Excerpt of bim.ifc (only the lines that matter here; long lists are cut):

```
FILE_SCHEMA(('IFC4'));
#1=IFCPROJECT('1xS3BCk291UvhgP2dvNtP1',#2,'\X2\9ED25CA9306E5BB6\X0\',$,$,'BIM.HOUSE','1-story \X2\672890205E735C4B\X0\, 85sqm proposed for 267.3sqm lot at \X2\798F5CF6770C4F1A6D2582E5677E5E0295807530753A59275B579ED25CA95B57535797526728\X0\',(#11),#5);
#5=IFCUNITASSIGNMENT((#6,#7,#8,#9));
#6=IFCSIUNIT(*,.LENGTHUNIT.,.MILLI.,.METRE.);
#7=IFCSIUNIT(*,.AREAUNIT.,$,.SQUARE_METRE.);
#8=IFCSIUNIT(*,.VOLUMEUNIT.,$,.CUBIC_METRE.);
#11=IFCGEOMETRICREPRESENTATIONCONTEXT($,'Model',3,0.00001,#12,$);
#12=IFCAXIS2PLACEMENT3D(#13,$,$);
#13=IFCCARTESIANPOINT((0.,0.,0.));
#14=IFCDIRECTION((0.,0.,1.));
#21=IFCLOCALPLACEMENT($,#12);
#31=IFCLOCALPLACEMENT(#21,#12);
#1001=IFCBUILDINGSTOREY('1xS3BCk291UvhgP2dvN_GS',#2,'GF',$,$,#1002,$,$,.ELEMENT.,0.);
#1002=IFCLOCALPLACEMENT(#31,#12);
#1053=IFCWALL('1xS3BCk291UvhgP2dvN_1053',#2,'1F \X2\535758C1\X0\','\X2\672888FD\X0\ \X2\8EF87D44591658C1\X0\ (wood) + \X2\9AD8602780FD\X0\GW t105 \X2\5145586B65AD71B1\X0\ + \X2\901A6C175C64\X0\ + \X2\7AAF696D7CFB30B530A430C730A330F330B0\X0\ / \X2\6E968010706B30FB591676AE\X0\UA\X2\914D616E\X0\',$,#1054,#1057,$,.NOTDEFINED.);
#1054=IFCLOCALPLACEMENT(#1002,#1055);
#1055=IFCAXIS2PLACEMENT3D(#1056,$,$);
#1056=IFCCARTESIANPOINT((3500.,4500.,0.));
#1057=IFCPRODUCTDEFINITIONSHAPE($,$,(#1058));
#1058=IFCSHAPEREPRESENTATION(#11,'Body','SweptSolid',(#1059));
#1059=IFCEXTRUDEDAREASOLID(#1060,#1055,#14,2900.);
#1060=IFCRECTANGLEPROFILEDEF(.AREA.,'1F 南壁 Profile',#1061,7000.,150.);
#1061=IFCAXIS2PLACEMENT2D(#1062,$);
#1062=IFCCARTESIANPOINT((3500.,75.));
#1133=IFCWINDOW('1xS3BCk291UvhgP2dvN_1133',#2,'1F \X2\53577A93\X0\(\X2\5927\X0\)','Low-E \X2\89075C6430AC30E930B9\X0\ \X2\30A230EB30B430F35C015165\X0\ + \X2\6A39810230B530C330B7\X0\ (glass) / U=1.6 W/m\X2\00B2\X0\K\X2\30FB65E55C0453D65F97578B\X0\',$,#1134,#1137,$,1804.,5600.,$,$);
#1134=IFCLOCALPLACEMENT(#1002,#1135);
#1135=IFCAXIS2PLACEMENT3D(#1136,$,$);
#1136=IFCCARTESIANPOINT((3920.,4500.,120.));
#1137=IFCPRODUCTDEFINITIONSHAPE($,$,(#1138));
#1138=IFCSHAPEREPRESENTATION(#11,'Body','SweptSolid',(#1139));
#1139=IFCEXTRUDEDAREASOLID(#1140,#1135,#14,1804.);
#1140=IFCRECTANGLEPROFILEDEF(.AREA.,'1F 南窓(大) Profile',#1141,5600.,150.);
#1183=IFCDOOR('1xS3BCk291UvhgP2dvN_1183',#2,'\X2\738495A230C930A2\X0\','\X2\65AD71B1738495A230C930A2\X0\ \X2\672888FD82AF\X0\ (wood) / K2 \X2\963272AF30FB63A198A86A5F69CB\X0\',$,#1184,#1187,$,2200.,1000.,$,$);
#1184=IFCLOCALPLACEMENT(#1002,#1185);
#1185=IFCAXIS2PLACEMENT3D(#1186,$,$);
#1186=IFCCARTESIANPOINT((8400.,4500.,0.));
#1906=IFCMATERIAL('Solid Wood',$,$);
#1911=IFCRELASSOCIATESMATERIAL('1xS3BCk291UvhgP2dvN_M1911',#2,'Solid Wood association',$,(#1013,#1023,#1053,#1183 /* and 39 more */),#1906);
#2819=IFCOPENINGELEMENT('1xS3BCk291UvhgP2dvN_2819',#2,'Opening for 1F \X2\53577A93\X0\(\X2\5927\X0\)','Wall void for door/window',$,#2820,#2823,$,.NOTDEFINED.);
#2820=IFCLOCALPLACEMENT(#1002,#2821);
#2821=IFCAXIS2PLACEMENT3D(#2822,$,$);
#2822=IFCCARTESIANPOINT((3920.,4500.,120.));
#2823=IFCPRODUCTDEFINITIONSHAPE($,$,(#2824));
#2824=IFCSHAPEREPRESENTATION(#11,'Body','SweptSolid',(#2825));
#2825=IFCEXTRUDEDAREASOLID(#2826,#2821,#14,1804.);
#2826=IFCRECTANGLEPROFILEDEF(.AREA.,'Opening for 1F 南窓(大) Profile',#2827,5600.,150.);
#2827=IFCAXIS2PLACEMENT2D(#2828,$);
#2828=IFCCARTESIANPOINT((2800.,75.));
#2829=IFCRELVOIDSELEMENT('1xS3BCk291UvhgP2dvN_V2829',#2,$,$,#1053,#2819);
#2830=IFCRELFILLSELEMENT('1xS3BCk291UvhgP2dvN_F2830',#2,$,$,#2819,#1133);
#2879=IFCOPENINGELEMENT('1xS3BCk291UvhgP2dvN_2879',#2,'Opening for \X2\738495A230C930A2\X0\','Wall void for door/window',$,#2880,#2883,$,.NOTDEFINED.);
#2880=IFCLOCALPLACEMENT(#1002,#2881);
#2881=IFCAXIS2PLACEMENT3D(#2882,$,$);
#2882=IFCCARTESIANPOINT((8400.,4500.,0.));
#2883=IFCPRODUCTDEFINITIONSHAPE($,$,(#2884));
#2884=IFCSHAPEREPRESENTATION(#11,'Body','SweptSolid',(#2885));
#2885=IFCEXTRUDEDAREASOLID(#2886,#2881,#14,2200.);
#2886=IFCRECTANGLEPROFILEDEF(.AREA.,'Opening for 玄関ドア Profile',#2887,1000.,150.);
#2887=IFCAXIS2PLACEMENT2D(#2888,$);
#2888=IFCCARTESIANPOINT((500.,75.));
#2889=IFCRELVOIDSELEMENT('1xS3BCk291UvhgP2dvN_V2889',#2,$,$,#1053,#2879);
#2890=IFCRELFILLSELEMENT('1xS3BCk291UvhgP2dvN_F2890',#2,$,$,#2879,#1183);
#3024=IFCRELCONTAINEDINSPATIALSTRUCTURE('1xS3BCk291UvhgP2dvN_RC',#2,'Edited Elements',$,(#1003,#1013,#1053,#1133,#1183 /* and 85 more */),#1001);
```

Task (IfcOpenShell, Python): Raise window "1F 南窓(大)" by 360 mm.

```python
import numpy as np
import ifcopenshell
import ifcopenshell.api.geometry
import ifcopenshell.util.placement
import ifcopenshell.util.unit

model = ifcopenshell.open("bim.ifc")
unit_scale = ifcopenshell.util.unit.calculate_unit_scale(model)

window = model.by_guid("1xS3BCk291UvhgP2dvN_1133")
opening = window.FillsVoids[0].RelatingOpeningElement
dz = 0.36 / unit_scale

shift = np.array([0.0, 0.0, dz])
# The window is not placed relative to its opening, so move both.
for product in (opening, window):
    matrix = ifcopenshell.util.placement.get_local_placement(product.ObjectPlacement)
    matrix[:3, 3] += shift
    ifcopenshell.api.geometry.edit_object_placement(model, product=product, matrix=matrix, is_si=False)

print(f"moved by {dz * unit_scale:+.3f} m")

model.write("bim_v2.ifc")
```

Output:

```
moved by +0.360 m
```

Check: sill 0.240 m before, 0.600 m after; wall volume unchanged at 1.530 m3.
